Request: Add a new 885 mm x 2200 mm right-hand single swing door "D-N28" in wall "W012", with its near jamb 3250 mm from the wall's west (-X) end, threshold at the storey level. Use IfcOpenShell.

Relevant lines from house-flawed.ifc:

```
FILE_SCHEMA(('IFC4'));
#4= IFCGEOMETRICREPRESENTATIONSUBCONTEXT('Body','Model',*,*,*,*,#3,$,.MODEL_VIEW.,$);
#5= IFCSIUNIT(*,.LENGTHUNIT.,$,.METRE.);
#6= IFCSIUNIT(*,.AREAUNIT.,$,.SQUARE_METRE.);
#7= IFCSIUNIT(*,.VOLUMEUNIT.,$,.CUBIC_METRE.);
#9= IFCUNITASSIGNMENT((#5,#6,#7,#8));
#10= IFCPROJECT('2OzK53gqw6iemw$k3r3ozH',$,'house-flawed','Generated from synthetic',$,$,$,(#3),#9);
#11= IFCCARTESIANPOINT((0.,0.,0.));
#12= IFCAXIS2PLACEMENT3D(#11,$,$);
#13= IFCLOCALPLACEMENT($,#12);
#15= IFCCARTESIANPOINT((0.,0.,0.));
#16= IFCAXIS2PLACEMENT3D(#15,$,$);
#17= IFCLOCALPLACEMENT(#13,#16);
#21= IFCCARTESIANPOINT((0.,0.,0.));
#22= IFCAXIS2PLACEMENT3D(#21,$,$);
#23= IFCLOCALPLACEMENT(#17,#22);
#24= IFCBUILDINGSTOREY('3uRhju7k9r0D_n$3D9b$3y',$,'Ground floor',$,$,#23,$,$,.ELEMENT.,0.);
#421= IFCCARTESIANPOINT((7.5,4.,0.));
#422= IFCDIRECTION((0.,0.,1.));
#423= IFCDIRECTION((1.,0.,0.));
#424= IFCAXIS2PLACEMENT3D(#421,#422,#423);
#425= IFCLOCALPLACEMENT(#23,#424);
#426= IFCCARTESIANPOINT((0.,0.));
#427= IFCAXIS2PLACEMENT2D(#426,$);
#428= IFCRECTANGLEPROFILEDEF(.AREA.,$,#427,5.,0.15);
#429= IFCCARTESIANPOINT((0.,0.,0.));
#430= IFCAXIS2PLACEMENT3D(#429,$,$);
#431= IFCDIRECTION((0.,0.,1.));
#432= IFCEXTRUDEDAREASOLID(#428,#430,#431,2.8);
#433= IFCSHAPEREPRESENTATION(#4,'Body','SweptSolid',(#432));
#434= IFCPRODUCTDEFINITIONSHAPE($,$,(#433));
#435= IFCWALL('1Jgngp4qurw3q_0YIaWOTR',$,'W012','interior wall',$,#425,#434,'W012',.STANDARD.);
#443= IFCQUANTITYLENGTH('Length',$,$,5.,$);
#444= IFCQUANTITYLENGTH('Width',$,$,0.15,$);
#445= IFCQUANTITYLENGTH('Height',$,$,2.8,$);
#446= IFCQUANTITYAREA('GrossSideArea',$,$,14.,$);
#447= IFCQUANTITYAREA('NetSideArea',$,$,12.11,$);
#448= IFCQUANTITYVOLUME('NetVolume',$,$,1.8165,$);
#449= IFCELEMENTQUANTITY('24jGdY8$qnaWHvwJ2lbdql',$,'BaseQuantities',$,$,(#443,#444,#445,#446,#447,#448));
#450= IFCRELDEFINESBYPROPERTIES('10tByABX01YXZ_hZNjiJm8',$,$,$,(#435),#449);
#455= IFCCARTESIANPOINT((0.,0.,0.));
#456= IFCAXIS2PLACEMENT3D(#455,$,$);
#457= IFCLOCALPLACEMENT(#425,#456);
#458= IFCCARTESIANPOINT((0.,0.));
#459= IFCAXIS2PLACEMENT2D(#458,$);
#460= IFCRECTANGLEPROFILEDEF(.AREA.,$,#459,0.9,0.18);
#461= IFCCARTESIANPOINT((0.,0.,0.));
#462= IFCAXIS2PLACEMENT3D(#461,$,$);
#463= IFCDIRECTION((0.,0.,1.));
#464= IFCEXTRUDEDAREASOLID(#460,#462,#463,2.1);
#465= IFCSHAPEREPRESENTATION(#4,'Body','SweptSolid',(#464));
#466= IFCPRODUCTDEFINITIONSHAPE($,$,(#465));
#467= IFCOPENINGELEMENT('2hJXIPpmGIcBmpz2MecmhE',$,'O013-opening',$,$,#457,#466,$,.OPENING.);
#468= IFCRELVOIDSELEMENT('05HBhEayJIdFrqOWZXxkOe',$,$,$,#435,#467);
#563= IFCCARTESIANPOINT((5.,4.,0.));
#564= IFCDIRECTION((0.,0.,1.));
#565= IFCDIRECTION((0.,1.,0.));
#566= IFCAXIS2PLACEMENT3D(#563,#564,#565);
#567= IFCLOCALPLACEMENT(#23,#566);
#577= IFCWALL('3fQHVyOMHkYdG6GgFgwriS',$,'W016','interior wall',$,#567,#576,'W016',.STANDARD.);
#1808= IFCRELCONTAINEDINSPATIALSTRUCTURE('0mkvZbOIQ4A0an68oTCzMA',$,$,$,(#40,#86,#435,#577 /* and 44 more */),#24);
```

```python
import numpy as np
import ifcopenshell
import ifcopenshell.api.feature
import ifcopenshell.api.geometry
import ifcopenshell.api.pset
import ifcopenshell.api.root
import ifcopenshell.api.spatial
import ifcopenshell.geom
import ifcopenshell.util.element
import ifcopenshell.util.placement
import ifcopenshell.util.representation
import ifcopenshell.util.shape
import ifcopenshell.util.unit

model = ifcopenshell.open("house-flawed.ifc")
unit_scale = ifcopenshell.util.unit.calculate_unit_scale(model)
area_scale = ifcopenshell.util.unit.calculate_unit_scale(model, "AREAUNIT")
volume_scale = ifcopenshell.util.unit.calculate_unit_scale(model, "VOLUMEUNIT")
settings = ifcopenshell.geom.settings()


def volume(element):
    """Net volume in cubic metres, openings subtracted."""
    shape = ifcopenshell.geom.create_shape(settings, element)
    return ifcopenshell.util.shape.get_volume(shape.geometry)


wall = model.by_guid("1Jgngp4qurw3q_0YIaWOTR")
storey = ifcopenshell.util.element.get_container(wall, ifc_class="IfcBuildingStorey")
context = ifcopenshell.util.representation.get_context(model, "Model", "Body", "MODEL_VIEW")
before = volume(wall)

width, height, from_end, sill = 0.885, 2.2, 3.25, 0.0  # metres

# The wall runs along its own X axis, and the end named is its -X end.
wall_shape = ifcopenshell.geom.create_shape(settings, wall)
x, y, z = ifcopenshell.util.shape.get_vertices(wall_shape.geometry).T
start = x.min() + from_end
face, thickness = float(y.min()), float(y.max() - y.min())
wall_matrix = ifcopenshell.util.placement.get_local_placement(wall.ObjectPlacement)
level = ifcopenshell.util.placement.get_local_placement(storey.ObjectPlacement)[2, 3]


def in_wall(x, y):
    """Placement at x, y metres in the wall's axes, at sill height."""
    matrix = wall_matrix.copy()
    matrix[:, 3] = wall_matrix @ np.array([x / unit_scale, y / unit_scale, 0.0, 1.0])
    matrix[2, 3] = level + sill / unit_scale
    return matrix


# Opening: a box that overshoots both wall faces by 50 mm.
opening = ifcopenshell.api.root.create_entity(model, ifc_class="IfcOpeningElement", predefined_type="OPENING")
box = ifcopenshell.api.geometry.add_wall_representation(
    model, context=context, length=width, height=height, thickness=thickness + 0.1
)
ifcopenshell.api.geometry.assign_representation(model, product=opening, representation=box)
ifcopenshell.api.geometry.edit_object_placement(model, product=opening, matrix=in_wall(start, face - 0.05), is_si=False)
ifcopenshell.api.feature.add_feature(model, feature=opening, element=wall)

door = ifcopenshell.api.root.create_entity(model, ifc_class="IfcDoor", name="D-N28", predefined_type="DOOR")
door.OverallWidth, door.OverallHeight = width / unit_scale, height / unit_scale
door.OperationType = "SINGLE_SWING_RIGHT"
body = ifcopenshell.api.geometry.add_door_representation(
    model,
    context=context,
    overall_width=door.OverallWidth,
    overall_height=door.OverallHeight,
    operation_type="SINGLE_SWING_RIGHT",
    lining_properties={"LiningDepth": thickness / unit_scale, "ThresholdDepth": thickness / unit_scale},
)
ifcopenshell.api.geometry.assign_representation(model, product=door, representation=body)
ifcopenshell.api.spatial.assign_container(model, products=[door], relating_structure=storey)
ifcopenshell.api.feature.add_filling(model, opening=opening, element=door)

# The lining spans the wall, so the door starts at the wall face.
ifcopenshell.api.geometry.edit_object_placement(model, product=door, matrix=in_wall(start, face), is_si=False)

after = volume(wall)

# Update the wall's stored quantities.
qto = model.by_id(ifcopenshell.util.element.get_pset(wall, "BaseQuantities", should_inherit=False)["id"])
ifcopenshell.api.pset.edit_qto(model, qto=qto, properties={
    "NetSideArea": after / thickness / area_scale,
    "NetVolume": after / volume_scale,
})

print(f"wall volume {before:.3f} -> {after:.3f} m3")

model.write("house-flawed_rev.ifc")
```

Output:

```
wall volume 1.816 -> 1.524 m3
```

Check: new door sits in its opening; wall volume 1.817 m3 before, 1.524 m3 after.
